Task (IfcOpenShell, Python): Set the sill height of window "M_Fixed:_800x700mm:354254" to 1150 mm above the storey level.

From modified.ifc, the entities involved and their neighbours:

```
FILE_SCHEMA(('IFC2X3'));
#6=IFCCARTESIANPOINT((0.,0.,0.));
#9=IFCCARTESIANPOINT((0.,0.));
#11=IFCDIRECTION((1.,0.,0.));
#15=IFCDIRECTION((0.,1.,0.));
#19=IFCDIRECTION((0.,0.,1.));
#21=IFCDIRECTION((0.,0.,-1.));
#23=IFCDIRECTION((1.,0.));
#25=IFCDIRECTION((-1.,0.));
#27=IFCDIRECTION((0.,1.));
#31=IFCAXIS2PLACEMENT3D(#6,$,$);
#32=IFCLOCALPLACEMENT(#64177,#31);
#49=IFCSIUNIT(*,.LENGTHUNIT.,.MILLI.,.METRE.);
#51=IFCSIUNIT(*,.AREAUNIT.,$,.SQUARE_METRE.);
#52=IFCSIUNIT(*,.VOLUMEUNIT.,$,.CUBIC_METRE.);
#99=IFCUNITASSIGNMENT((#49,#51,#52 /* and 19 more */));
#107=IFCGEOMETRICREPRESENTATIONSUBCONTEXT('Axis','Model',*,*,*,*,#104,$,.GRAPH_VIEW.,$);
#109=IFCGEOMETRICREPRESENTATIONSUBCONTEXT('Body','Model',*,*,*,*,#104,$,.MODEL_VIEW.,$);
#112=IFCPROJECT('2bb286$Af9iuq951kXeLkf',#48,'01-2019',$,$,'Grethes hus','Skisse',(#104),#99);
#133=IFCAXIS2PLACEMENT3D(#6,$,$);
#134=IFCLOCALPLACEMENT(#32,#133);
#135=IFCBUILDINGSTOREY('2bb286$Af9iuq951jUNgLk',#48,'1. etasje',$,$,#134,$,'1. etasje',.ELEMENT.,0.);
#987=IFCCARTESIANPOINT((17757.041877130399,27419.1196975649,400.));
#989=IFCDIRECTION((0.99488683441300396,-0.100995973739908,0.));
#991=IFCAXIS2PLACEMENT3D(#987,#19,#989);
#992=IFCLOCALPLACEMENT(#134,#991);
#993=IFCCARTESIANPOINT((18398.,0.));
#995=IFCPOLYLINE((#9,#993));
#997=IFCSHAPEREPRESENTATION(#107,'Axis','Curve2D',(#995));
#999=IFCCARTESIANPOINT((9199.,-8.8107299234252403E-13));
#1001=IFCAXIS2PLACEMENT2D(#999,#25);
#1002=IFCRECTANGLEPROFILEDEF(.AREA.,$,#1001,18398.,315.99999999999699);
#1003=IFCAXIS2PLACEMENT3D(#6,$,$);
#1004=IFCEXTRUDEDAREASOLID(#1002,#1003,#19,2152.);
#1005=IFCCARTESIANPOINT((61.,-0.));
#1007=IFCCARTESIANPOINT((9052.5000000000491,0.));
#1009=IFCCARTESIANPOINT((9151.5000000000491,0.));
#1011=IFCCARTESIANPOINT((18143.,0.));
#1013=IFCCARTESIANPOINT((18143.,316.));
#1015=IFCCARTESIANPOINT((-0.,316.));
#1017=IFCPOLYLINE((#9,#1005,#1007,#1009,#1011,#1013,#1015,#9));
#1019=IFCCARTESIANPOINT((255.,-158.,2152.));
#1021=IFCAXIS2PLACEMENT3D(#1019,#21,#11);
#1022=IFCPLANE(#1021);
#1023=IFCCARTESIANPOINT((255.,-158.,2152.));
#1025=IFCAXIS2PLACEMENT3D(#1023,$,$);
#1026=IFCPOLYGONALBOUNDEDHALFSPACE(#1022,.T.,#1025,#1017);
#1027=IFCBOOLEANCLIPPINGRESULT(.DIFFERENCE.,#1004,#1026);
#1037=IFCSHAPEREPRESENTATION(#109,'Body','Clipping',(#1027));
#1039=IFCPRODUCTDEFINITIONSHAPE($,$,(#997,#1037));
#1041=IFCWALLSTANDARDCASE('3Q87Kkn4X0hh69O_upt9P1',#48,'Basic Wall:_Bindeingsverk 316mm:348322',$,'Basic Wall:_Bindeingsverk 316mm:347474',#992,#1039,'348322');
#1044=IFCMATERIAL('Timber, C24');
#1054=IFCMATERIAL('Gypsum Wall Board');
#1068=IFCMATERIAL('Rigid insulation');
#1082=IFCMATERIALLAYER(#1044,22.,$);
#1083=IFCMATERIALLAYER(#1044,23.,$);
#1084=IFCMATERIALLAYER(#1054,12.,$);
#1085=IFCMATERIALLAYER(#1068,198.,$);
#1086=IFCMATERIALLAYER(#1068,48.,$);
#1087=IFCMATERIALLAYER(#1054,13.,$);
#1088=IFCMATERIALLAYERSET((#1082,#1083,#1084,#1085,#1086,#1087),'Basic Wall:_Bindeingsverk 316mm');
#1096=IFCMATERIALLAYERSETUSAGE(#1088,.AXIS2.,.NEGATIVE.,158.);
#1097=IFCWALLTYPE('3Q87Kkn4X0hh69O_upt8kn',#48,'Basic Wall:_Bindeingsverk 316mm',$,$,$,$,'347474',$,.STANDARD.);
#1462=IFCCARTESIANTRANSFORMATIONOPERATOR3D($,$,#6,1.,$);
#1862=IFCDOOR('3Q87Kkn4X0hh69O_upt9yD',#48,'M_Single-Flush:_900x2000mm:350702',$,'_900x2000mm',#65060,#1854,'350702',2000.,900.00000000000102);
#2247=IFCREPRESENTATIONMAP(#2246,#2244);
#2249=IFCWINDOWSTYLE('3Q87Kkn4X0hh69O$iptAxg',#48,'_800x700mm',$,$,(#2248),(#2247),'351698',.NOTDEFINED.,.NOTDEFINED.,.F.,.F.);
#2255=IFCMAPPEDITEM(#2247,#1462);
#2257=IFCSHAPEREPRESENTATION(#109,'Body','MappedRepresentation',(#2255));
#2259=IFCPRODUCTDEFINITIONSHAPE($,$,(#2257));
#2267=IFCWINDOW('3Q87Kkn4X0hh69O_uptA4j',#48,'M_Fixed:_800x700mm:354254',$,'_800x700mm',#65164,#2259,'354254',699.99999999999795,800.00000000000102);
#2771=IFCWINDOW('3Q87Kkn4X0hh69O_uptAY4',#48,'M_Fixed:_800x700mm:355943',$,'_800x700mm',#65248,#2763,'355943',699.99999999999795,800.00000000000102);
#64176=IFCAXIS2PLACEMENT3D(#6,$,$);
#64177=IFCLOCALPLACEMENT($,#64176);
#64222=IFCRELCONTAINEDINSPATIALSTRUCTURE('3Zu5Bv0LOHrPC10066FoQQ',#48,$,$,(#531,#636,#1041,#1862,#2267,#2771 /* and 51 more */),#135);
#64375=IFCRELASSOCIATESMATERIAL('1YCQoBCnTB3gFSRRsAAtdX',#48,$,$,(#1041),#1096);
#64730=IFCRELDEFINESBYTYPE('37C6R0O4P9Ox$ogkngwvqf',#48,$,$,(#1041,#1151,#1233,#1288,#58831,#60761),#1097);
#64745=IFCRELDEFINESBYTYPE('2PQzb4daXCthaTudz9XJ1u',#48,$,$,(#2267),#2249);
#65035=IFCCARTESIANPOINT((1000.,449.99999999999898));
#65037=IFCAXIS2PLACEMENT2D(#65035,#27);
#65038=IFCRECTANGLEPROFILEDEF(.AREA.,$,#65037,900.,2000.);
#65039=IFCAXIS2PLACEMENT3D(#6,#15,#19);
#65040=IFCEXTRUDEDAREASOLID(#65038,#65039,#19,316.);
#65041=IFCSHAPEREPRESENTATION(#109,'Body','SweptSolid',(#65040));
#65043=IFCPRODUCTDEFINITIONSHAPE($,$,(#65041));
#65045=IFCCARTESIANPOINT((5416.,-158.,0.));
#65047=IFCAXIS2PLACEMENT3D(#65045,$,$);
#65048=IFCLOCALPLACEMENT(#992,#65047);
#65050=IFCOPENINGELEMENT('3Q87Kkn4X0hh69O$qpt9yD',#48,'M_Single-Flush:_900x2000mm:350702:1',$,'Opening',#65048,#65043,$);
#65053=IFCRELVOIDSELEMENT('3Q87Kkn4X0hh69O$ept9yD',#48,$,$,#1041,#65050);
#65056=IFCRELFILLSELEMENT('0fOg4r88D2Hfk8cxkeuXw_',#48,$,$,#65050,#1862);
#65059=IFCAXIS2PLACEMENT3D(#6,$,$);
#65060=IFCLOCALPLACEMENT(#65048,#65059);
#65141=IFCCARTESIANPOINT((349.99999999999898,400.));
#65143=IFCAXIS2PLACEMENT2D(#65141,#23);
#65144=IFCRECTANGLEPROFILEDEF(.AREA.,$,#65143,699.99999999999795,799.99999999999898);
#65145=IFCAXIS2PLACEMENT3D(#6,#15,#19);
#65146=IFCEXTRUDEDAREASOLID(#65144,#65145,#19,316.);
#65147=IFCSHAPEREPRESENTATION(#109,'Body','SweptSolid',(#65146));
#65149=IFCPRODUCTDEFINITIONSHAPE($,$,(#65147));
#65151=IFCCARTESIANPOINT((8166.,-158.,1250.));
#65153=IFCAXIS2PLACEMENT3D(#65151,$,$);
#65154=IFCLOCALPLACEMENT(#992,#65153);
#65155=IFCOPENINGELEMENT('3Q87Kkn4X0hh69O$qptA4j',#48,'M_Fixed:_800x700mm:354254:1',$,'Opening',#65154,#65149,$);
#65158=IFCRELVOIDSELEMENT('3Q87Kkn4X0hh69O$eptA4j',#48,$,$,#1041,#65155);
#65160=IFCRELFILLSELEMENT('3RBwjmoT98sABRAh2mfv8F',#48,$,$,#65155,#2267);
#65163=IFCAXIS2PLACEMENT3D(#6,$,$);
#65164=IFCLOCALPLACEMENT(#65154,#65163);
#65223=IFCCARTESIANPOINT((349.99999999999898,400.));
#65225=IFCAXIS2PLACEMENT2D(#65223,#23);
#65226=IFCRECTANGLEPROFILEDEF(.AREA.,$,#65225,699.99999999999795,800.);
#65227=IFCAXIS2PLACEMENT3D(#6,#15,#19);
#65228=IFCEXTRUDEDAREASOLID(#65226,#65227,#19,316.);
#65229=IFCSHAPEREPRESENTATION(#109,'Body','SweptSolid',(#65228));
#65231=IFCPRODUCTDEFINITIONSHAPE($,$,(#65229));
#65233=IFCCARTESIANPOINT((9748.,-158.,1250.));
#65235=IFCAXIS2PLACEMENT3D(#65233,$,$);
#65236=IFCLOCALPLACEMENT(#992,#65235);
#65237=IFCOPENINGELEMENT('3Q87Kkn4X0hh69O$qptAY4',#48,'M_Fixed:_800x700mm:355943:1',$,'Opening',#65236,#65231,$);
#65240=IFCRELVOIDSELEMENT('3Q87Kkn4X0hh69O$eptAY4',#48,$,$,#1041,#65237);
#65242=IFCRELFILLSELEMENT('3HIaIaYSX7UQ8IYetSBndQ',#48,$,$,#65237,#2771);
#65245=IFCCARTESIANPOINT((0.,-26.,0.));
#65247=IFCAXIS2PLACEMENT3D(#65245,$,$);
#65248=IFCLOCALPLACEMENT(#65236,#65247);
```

```python
import numpy as np
import ifcopenshell
import ifcopenshell.api.geometry
import ifcopenshell.geom
import ifcopenshell.util.element
import ifcopenshell.util.placement
import ifcopenshell.util.shape
import ifcopenshell.util.unit

model = ifcopenshell.open("modified.ifc")
unit_scale = ifcopenshell.util.unit.calculate_unit_scale(model)

window = model.by_guid("3Q87Kkn4X0hh69O_uptA4j")
opening = window.FillsVoids[0].RelatingOpeningElement
storey = ifcopenshell.util.element.get_container(window, ifc_class="IfcBuildingStorey")
level = ifcopenshell.util.placement.get_local_placement(storey.ObjectPlacement)[2, 3]

# The opening's origin need not be at the sill, so measure its lowest point.
shape = ifcopenshell.geom.create_shape(ifcopenshell.geom.settings(), opening)
bottom = ifcopenshell.util.shape.get_shape_bottom_elevation(shape, shape.geometry) / unit_scale
dz = level + 1150.0 - bottom

shift = np.array([0.0, 0.0, dz])
# The window is placed relative to its opening, so it follows when the opening moves.
matrix = ifcopenshell.util.placement.get_local_placement(opening.ObjectPlacement)
matrix[:3, 3] += shift
ifcopenshell.api.geometry.edit_object_placement(
    model, product=opening, matrix=matrix, is_si=False, should_transform_children=True
)

print(f"moved by {dz * unit_scale:+.3f} m")

model.write("modified_updated.ifc")
```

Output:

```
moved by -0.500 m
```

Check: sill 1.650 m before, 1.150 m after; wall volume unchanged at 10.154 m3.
